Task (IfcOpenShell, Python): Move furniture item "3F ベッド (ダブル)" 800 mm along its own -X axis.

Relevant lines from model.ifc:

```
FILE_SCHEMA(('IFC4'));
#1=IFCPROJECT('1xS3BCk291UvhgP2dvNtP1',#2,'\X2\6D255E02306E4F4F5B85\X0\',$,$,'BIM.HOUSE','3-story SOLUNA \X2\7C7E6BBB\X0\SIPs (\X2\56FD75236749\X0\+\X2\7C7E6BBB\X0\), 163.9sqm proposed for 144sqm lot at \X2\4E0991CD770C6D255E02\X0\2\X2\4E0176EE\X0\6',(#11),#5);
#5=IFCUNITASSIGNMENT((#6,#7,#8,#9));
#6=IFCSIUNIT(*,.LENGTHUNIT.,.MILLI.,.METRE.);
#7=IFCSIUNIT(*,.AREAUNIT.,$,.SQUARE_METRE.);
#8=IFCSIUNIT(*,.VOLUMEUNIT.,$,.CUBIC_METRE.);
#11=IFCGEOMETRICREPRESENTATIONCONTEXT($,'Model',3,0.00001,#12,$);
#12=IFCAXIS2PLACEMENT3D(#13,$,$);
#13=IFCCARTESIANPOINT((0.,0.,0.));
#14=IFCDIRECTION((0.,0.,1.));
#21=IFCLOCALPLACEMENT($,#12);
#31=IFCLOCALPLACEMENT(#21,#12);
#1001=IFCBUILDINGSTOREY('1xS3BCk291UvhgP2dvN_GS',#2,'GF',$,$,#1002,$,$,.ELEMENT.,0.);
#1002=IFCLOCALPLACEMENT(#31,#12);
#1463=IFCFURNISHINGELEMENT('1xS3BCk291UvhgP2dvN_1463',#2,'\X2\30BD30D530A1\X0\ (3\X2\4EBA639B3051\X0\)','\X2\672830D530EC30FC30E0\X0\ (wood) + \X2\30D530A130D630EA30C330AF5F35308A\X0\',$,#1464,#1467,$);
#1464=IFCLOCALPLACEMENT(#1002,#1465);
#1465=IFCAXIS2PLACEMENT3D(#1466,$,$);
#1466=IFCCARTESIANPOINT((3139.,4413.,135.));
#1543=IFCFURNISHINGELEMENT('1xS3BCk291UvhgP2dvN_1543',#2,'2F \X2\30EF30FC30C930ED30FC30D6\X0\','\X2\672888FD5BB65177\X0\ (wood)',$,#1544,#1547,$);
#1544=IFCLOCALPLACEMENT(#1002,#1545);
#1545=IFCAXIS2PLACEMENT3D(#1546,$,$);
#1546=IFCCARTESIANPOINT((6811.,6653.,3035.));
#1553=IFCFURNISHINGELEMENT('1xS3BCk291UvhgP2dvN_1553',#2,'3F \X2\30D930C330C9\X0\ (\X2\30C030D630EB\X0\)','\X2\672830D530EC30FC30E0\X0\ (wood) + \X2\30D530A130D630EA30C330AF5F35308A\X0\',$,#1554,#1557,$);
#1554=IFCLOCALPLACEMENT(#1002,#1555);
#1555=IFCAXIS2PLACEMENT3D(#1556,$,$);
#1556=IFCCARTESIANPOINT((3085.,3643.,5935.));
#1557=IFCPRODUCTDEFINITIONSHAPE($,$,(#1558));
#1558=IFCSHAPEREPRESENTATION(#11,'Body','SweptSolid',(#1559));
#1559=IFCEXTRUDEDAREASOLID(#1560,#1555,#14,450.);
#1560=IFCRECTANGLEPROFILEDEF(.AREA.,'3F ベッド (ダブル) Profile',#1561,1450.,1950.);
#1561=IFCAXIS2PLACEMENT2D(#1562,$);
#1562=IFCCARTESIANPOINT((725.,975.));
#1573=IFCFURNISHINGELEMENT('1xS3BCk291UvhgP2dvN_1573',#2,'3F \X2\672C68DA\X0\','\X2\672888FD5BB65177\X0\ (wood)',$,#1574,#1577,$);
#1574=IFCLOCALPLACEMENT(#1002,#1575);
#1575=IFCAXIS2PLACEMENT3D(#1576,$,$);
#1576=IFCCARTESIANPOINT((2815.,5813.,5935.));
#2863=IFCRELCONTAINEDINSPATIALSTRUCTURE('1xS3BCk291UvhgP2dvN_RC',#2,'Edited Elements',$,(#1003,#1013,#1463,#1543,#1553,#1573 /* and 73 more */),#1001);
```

```python
import ifcopenshell
import ifcopenshell.api.geometry
import ifcopenshell.util.placement

model = ifcopenshell.open("model.ifc")

item = model.by_id(1553)
matrix = ifcopenshell.util.placement.get_local_placement(item.ObjectPlacement)
matrix[:3, 3] -= matrix[:3, 0] * 800.0
ifcopenshell.api.geometry.edit_object_placement(model, product=item, matrix=matrix, is_si=False)

print(ifcopenshell.util.placement.get_local_placement(item.ObjectPlacement).round(3) + 0.0)

model.write("model_updated.ifc")
```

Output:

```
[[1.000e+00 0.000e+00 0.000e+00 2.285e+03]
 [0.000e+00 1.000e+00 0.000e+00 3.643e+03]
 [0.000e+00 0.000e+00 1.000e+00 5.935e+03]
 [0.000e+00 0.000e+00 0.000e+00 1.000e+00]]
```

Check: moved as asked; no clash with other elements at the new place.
